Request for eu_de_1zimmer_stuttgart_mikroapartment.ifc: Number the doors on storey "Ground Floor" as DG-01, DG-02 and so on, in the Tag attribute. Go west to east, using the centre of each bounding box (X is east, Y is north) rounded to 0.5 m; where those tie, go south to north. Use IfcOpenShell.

First a look at what the model holds.

```python
import ifcopenshell
import ifcopenshell.util.element
import ifcopenshell.util.placement

model = ifcopenshell.open("eu_de_1zimmer_stuttgart_mikroapartment.ifc")
print(model.schema)
storey = next(s for s in model.by_type("IfcBuildingStorey") if s.Name == "Ground Floor")
doors = [e for e in ifcopenshell.util.element.get_decomposition(storey) if e.is_a("IfcDoor")]
for e in sorted(doors, key=lambda e: e.id()):
    origin = ifcopenshell.util.placement.get_local_placement(e.ObjectPlacement)[:3, 3]
    print(e.id(), e.Tag, e.Name, origin.round(2) + 0.0, sep=" | ")
```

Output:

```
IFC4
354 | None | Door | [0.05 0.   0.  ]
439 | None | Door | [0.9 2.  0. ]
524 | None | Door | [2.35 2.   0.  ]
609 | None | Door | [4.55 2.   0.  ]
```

```python
import ifcopenshell
import ifcopenshell.geom
import ifcopenshell.util.element
import ifcopenshell.util.shape

model = ifcopenshell.open("eu_de_1zimmer_stuttgart_mikroapartment.ifc")
settings = ifcopenshell.geom.settings()
settings.set("use-world-coords", True)


def centre(element):
    shape = ifcopenshell.geom.create_shape(settings, element)
    return ifcopenshell.util.shape.get_bbox_centroid(shape.geometry)


storey = next(s for s in model.by_type("IfcBuildingStorey") if s.Name == "Ground Floor")
doors = [e for e in ifcopenshell.util.element.get_decomposition(storey) if e.is_a("IfcDoor")]

# Insertion points can sit at a corner or the storey origin, so sort by the geometry (in metres).
centres = {e: centre(e) for e in doors}
doors.sort(key=lambda e: (round(centres[e][0] / 0.5), centres[e][1]))

for i, e in enumerate(doors, start=1):
    number = f"DG-{i:02d}"
    e.Tag = number
    print(e.id(), number)

model.write("eu_de_1zimmer_stuttgart_mikroapartment_edited.ifc")
```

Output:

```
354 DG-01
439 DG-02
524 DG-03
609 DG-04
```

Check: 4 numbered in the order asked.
